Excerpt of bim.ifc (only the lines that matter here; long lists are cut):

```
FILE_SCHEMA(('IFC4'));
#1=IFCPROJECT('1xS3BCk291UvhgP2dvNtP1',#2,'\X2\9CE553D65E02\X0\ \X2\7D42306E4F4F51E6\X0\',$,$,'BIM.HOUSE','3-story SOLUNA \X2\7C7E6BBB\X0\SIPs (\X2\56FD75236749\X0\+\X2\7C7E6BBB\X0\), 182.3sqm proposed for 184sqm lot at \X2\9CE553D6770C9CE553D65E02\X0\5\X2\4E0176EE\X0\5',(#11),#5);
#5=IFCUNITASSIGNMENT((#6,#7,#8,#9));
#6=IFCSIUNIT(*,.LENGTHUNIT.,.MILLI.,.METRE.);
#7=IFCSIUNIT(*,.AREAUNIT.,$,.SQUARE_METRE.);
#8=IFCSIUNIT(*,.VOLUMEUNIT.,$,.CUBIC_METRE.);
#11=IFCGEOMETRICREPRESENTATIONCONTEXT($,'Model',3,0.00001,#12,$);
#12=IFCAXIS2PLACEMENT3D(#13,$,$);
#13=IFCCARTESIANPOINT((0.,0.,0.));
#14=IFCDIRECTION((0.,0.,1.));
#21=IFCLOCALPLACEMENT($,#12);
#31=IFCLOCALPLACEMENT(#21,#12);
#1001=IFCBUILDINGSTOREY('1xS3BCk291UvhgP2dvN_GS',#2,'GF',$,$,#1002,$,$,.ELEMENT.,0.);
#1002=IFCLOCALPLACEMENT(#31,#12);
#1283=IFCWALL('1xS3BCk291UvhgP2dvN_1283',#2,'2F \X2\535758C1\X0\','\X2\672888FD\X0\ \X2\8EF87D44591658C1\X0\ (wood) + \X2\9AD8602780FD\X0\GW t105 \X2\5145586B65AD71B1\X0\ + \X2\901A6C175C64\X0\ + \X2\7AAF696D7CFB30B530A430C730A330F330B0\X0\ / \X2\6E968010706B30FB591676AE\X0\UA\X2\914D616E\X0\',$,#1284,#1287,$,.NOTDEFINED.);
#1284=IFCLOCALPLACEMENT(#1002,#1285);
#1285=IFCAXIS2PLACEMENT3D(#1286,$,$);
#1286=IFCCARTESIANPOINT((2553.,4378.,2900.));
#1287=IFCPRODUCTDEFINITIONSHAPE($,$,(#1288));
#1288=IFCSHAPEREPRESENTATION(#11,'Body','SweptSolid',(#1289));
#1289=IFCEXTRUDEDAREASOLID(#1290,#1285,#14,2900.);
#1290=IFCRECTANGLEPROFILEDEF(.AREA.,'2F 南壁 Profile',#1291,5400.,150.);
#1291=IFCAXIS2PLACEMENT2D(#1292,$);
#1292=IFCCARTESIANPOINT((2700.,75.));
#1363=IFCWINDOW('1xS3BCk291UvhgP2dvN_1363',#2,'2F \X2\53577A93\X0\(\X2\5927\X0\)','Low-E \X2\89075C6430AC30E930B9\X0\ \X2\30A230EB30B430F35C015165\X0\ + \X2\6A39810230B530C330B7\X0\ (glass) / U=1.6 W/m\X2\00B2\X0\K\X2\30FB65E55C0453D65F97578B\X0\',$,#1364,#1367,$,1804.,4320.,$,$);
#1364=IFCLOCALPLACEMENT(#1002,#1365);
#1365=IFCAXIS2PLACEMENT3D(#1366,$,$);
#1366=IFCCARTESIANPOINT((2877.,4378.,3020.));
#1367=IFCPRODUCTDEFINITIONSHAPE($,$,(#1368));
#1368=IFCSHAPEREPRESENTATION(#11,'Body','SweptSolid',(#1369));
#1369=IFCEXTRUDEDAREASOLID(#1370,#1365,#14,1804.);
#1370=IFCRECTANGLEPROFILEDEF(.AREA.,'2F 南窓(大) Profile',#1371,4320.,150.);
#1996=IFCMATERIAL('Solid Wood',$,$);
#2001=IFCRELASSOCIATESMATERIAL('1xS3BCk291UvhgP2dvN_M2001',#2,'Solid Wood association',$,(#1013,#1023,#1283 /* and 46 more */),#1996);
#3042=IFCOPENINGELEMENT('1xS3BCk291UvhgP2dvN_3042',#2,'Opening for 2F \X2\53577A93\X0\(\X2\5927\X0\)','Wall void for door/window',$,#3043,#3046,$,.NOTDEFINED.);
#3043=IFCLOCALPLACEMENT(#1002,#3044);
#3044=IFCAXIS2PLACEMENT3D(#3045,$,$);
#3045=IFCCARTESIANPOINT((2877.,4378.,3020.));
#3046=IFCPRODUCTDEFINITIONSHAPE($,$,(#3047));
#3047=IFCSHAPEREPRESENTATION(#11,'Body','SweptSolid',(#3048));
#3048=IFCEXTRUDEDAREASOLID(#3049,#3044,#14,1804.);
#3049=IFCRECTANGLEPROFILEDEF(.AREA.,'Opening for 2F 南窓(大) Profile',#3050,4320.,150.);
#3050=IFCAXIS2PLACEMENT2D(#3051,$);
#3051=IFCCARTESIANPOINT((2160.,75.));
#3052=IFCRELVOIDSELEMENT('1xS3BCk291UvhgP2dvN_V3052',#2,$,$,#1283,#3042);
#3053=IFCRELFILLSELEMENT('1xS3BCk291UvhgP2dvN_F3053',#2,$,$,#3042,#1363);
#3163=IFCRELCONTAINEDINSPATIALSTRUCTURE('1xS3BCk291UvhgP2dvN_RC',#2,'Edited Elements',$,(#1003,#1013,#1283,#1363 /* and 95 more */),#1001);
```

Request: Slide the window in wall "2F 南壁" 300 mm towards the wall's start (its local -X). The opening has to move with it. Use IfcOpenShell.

```python
import ifcopenshell
import ifcopenshell.api.geometry
import ifcopenshell.util.placement
import ifcopenshell.util.unit

model = ifcopenshell.open("bim.ifc")
unit_scale = ifcopenshell.util.unit.calculate_unit_scale(model)

window = model.by_guid("1xS3BCk291UvhgP2dvN_1363")
opening = window.FillsVoids[0].RelatingOpeningElement
wall = opening.VoidsElements[0].RelatingBuildingElement

wall_matrix = ifcopenshell.util.placement.get_local_placement(wall.ObjectPlacement)
shift = wall_matrix[:3, 0] * -0.3 / unit_scale
before = ifcopenshell.util.placement.get_local_placement(window.ObjectPlacement)[:3, 3].copy()

# The window is not placed relative to its opening, so move both.
for product in (opening, window):
    matrix = ifcopenshell.util.placement.get_local_placement(product.ObjectPlacement)
    matrix[:3, 3] += shift
    ifcopenshell.api.geometry.edit_object_placement(model, product=product, matrix=matrix, is_si=False)

after = ifcopenshell.util.placement.get_local_placement(window.ObjectPlacement)[:3, 3]
print("window moved by", (after - before).round(3) + 0.0)

model.write("bim_updated.ifc")
```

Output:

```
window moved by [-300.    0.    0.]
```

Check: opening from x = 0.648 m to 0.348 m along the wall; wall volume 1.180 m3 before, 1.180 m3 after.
